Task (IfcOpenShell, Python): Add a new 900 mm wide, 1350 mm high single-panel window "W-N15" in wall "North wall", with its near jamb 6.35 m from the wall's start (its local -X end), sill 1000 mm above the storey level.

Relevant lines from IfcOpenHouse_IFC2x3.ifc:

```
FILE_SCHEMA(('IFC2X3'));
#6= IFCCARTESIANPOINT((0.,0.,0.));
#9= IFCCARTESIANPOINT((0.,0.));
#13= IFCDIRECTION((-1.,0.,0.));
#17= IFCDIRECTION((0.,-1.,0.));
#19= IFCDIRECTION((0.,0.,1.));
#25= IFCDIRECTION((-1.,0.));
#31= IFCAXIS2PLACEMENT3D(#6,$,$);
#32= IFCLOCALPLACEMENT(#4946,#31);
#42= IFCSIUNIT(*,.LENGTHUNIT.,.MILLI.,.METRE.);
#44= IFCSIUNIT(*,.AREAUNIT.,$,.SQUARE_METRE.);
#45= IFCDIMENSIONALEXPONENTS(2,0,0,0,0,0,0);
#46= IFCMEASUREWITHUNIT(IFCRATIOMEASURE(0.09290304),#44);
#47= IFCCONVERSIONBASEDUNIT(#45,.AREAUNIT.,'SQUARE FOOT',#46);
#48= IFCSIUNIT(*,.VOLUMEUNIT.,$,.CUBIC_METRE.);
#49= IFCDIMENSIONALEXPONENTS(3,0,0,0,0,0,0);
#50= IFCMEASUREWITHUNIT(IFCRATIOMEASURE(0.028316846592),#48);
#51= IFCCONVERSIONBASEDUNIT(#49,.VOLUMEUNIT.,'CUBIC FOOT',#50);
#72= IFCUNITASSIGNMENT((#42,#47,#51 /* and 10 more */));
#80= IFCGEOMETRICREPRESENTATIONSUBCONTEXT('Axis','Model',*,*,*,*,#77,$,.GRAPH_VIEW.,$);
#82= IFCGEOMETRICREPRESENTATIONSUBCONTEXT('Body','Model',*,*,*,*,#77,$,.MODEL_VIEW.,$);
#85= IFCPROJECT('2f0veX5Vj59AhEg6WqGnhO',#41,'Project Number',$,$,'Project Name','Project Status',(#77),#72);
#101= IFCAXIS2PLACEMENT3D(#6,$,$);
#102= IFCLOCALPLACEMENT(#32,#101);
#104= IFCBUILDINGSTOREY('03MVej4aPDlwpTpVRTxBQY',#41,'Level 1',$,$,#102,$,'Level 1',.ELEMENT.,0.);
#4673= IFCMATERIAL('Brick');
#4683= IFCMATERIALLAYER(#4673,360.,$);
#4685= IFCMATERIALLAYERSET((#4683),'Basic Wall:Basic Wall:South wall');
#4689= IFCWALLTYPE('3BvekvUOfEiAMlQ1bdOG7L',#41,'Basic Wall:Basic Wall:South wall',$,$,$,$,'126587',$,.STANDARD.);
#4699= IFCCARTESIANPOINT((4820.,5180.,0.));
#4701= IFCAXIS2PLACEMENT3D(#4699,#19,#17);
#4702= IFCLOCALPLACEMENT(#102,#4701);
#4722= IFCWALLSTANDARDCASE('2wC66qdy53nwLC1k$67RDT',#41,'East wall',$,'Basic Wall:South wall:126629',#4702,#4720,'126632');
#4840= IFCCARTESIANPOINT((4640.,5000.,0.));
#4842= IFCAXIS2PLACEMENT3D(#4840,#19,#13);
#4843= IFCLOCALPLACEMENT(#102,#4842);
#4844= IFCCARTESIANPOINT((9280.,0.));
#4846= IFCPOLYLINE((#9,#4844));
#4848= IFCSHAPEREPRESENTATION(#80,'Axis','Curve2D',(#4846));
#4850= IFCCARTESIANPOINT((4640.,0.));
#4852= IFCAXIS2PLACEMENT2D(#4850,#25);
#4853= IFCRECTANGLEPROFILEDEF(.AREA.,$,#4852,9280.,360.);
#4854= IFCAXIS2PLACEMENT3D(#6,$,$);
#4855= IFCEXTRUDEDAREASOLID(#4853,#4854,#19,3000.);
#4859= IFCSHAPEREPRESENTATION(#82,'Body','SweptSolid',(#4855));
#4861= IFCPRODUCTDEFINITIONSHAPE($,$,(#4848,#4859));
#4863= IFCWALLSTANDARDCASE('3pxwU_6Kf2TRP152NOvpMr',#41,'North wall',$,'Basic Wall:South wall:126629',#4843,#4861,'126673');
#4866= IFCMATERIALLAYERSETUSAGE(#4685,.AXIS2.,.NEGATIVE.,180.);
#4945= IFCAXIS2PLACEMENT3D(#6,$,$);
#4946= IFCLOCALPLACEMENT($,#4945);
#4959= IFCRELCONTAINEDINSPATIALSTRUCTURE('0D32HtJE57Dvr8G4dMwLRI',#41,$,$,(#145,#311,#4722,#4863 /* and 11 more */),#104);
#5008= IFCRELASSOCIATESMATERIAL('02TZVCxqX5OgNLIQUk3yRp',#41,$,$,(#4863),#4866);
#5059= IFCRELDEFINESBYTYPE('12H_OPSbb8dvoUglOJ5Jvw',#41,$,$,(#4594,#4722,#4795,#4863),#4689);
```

```python
import numpy as np
import ifcopenshell
import ifcopenshell.api.feature
import ifcopenshell.api.geometry
import ifcopenshell.api.root
import ifcopenshell.api.spatial
import ifcopenshell.api.type
import ifcopenshell.geom
import ifcopenshell.util.element
import ifcopenshell.util.placement
import ifcopenshell.util.representation
import ifcopenshell.util.shape
import ifcopenshell.util.unit

model = ifcopenshell.open("IfcOpenHouse_IFC2x3.ifc")
unit_scale = ifcopenshell.util.unit.calculate_unit_scale(model)
settings = ifcopenshell.geom.settings()


def volume(element):
    """Net volume in cubic metres, openings subtracted."""
    shape = ifcopenshell.geom.create_shape(settings, element)
    return ifcopenshell.util.shape.get_volume(shape.geometry)


wall = model.by_guid("3pxwU_6Kf2TRP152NOvpMr")
storey = ifcopenshell.util.element.get_container(wall, ifc_class="IfcBuildingStorey")
context = ifcopenshell.util.representation.get_context(model, "Model", "Body", "MODEL_VIEW")
before = volume(wall)

width, height, from_end, sill = 0.9, 1.35, 6.35, 1  # metres

# The wall runs along its own X axis, and the end named is its -X end.
wall_shape = ifcopenshell.geom.create_shape(settings, wall)
x, y, z = ifcopenshell.util.shape.get_vertices(wall_shape.geometry).T
start = x.min() + from_end
face, thickness = float(y.min()), float(y.max() - y.min())
wall_matrix = ifcopenshell.util.placement.get_local_placement(wall.ObjectPlacement)
level = ifcopenshell.util.placement.get_local_placement(storey.ObjectPlacement)[2, 3]


def in_wall(x, y):
    """Placement at x, y metres in the wall's axes, at sill height."""
    matrix = wall_matrix.copy()
    matrix[:, 3] = wall_matrix @ np.array([x / unit_scale, y / unit_scale, 0.0, 1.0])
    matrix[2, 3] = level + sill / unit_scale
    return matrix


# Opening: a box that overshoots both wall faces by 50 mm.
opening = ifcopenshell.api.root.create_entity(model, ifc_class="IfcOpeningElement")
box = ifcopenshell.api.geometry.add_wall_representation(
    model, context=context, length=width, height=height, thickness=thickness + 0.1
)
ifcopenshell.api.geometry.assign_representation(model, product=opening, representation=box)
ifcopenshell.api.geometry.edit_object_placement(model, product=opening, matrix=in_wall(start, face - 0.05), is_si=False)
ifcopenshell.api.feature.add_feature(model, feature=opening, element=wall)

window = ifcopenshell.api.root.create_entity(model, ifc_class="IfcWindow", name="W-N15")
window.OverallWidth, window.OverallHeight = width / unit_scale, height / unit_scale
body = ifcopenshell.api.geometry.add_window_representation(
    model,
    context=context,
    overall_width=window.OverallWidth,
    overall_height=window.OverallHeight,
    partition_type="SINGLE_PANEL",
)
ifcopenshell.api.geometry.assign_representation(model, product=window, representation=body)
ifcopenshell.api.spatial.assign_container(model, products=[window], relating_structure=storey)
fills = ifcopenshell.api.feature.add_filling(model, opening=opening, element=window)
fills.OwnerHistory = window.OwnerHistory  # required in IFC2X3

# IFC2X3 keeps the operation on the window style.
style = ifcopenshell.api.root.create_entity(model, ifc_class="IfcWindowStyle", name="W-N15")
style.OperationType, style.ConstructionType = "SINGLE_PANEL", "NOTDEFINED"
style.ParameterTakesPrecedence = style.Sizeable = False
ifcopenshell.api.type.assign_type(model, related_objects=[window], relating_type=style)

# Centre the window in the wall's thickness.
ifcopenshell.api.geometry.edit_object_placement(model, product=window, matrix=in_wall(start, face), is_si=False)
window_shape = ifcopenshell.geom.create_shape(settings, window)
depth = ifcopenshell.util.shape.get_vertices(window_shape.geometry)[:, 1]
offset = face + thickness / 2 - (depth.min() + depth.max()) / 2
ifcopenshell.api.geometry.edit_object_placement(model, product=window, matrix=in_wall(start, offset), is_si=False)

after = volume(wall)

print(f"wall volume {before:.3f} -> {after:.3f} m3")

model.write("IfcOpenHouse_IFC2x3_v2.ifc")
```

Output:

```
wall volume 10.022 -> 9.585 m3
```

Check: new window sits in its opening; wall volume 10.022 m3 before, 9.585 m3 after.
